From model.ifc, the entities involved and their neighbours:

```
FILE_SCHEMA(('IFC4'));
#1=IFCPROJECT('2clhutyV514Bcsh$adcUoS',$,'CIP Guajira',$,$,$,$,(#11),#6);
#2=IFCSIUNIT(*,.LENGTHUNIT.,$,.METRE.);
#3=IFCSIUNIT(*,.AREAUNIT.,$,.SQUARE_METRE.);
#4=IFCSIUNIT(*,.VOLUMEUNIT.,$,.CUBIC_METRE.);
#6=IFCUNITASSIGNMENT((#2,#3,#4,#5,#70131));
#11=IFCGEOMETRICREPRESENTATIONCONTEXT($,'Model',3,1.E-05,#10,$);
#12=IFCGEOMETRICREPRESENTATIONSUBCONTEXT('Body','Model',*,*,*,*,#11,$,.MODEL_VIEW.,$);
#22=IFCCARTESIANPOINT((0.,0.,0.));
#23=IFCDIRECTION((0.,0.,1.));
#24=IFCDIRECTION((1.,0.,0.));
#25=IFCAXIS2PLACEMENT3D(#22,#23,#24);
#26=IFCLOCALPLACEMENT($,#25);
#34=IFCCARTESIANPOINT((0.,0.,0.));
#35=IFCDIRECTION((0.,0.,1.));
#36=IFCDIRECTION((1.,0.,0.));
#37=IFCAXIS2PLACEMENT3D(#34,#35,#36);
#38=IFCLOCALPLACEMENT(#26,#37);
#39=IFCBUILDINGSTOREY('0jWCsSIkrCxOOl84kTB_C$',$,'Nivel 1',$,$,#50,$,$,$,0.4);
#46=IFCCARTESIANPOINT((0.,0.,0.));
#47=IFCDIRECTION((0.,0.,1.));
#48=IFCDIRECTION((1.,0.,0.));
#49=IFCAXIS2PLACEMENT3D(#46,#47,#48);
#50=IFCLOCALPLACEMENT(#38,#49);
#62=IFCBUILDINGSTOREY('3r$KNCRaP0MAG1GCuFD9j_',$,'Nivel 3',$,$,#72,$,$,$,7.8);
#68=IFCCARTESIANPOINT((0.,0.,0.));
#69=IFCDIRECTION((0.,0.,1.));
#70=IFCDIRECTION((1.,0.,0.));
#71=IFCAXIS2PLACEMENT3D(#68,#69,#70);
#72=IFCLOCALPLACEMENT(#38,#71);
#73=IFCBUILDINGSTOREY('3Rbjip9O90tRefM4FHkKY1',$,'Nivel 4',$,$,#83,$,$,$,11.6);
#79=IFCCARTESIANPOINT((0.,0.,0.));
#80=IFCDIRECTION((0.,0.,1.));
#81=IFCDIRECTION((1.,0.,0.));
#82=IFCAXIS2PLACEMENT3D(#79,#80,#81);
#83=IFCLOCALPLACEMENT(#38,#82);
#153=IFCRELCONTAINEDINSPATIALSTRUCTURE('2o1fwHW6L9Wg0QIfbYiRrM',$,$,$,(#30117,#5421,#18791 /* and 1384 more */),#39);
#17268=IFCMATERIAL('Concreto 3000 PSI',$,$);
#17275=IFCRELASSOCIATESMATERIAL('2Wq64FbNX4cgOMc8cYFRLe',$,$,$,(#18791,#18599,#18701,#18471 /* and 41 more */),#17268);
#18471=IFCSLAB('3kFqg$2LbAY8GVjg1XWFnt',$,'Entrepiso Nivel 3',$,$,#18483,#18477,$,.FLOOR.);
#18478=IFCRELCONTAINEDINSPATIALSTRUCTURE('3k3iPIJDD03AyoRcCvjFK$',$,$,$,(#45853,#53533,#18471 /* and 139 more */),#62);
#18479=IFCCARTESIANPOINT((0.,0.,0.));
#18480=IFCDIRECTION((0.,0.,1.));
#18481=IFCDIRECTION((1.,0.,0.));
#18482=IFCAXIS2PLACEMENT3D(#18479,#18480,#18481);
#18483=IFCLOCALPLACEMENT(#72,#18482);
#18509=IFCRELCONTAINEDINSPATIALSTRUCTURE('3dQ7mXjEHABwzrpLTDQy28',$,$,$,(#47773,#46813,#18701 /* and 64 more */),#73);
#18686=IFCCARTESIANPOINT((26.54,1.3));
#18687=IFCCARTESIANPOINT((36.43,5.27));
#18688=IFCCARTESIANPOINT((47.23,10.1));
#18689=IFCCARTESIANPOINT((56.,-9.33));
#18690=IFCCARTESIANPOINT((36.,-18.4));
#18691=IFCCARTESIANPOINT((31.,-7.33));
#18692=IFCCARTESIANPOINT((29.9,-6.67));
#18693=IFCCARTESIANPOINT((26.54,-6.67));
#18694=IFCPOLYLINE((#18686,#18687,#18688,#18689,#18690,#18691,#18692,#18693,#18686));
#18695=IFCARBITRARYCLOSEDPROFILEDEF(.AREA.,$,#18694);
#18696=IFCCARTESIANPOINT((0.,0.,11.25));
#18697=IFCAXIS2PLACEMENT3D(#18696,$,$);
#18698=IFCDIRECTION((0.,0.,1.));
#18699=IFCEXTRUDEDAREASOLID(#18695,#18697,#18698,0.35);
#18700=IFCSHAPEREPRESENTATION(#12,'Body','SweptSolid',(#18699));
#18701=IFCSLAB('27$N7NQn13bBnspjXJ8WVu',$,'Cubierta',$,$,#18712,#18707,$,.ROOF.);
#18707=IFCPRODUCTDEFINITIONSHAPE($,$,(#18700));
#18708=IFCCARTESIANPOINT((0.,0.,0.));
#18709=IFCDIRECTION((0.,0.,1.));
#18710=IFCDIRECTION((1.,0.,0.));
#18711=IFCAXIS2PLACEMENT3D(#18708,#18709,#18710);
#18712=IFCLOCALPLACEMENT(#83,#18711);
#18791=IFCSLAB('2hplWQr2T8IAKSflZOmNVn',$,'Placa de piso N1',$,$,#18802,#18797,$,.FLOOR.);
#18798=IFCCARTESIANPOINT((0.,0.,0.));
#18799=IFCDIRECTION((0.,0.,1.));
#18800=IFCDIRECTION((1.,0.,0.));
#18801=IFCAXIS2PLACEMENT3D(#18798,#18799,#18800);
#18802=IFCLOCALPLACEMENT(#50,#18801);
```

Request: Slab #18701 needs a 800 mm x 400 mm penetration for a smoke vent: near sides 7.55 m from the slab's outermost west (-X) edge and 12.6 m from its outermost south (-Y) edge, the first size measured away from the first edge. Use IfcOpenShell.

```python
import numpy as np
import ifcopenshell
import ifcopenshell.api.feature
import ifcopenshell.api.geometry
import ifcopenshell.api.root
import ifcopenshell.geom
import ifcopenshell.util.placement
import ifcopenshell.util.representation
import ifcopenshell.util.shape
import ifcopenshell.util.unit

model = ifcopenshell.open("model.ifc")
unit_scale = ifcopenshell.util.unit.calculate_unit_scale(model)
settings = ifcopenshell.geom.settings()


def volume(element):
    """Net volume in cubic metres, openings subtracted."""
    shape = ifcopenshell.geom.create_shape(settings, element)
    return ifcopenshell.util.shape.get_volume(shape.geometry)


slab = model.by_guid("27$N7NQn13bBnspjXJ8WVu")
before = volume(slab)

# Extent in the slab's own axes, in metres. The edges named are its -X and -Y sides.
slab_shape = ifcopenshell.geom.create_shape(settings, slab)
vertices = ifcopenshell.util.shape.get_vertices(slab_shape.geometry)
x_min, y_min, bottom = vertices.min(axis=0)
top = vertices[:, 2].max()

opening = ifcopenshell.api.root.create_entity(model, ifc_class="IfcOpeningElement", name="Smoke vent opening", predefined_type="OPENING")
context = ifcopenshell.util.representation.get_context(model, "Model", "Body", "MODEL_VIEW")
width, depth = 0.8, 0.4
outline = [(0.0, 0.0), (width, 0.0), (width, depth), (0.0, depth), (0.0, 0.0)]
# Overshoot both faces by 50 mm so the cut is clean.
shape = ifcopenshell.api.geometry.add_slab_representation(
    model, context=context, depth=top - bottom + 0.1, polyline=outline
)
ifcopenshell.api.geometry.assign_representation(model, product=opening, representation=shape)

matrix = ifcopenshell.util.placement.get_local_placement(slab.ObjectPlacement)
matrix[:, 3] = matrix @ np.append(np.array([x_min + 7.55, y_min + 12.6, bottom - 0.05]) / unit_scale, 1.0)
ifcopenshell.api.geometry.edit_object_placement(model, product=opening, matrix=matrix, is_si=False)
ifcopenshell.api.feature.add_feature(model, feature=opening, element=slab)

after = volume(slab)

print(f"slab volume {before:.3f} -> {after:.3f} m3")

model.write("model-out.ifc")
```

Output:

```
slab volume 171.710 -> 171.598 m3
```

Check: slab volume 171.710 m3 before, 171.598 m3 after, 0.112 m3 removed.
